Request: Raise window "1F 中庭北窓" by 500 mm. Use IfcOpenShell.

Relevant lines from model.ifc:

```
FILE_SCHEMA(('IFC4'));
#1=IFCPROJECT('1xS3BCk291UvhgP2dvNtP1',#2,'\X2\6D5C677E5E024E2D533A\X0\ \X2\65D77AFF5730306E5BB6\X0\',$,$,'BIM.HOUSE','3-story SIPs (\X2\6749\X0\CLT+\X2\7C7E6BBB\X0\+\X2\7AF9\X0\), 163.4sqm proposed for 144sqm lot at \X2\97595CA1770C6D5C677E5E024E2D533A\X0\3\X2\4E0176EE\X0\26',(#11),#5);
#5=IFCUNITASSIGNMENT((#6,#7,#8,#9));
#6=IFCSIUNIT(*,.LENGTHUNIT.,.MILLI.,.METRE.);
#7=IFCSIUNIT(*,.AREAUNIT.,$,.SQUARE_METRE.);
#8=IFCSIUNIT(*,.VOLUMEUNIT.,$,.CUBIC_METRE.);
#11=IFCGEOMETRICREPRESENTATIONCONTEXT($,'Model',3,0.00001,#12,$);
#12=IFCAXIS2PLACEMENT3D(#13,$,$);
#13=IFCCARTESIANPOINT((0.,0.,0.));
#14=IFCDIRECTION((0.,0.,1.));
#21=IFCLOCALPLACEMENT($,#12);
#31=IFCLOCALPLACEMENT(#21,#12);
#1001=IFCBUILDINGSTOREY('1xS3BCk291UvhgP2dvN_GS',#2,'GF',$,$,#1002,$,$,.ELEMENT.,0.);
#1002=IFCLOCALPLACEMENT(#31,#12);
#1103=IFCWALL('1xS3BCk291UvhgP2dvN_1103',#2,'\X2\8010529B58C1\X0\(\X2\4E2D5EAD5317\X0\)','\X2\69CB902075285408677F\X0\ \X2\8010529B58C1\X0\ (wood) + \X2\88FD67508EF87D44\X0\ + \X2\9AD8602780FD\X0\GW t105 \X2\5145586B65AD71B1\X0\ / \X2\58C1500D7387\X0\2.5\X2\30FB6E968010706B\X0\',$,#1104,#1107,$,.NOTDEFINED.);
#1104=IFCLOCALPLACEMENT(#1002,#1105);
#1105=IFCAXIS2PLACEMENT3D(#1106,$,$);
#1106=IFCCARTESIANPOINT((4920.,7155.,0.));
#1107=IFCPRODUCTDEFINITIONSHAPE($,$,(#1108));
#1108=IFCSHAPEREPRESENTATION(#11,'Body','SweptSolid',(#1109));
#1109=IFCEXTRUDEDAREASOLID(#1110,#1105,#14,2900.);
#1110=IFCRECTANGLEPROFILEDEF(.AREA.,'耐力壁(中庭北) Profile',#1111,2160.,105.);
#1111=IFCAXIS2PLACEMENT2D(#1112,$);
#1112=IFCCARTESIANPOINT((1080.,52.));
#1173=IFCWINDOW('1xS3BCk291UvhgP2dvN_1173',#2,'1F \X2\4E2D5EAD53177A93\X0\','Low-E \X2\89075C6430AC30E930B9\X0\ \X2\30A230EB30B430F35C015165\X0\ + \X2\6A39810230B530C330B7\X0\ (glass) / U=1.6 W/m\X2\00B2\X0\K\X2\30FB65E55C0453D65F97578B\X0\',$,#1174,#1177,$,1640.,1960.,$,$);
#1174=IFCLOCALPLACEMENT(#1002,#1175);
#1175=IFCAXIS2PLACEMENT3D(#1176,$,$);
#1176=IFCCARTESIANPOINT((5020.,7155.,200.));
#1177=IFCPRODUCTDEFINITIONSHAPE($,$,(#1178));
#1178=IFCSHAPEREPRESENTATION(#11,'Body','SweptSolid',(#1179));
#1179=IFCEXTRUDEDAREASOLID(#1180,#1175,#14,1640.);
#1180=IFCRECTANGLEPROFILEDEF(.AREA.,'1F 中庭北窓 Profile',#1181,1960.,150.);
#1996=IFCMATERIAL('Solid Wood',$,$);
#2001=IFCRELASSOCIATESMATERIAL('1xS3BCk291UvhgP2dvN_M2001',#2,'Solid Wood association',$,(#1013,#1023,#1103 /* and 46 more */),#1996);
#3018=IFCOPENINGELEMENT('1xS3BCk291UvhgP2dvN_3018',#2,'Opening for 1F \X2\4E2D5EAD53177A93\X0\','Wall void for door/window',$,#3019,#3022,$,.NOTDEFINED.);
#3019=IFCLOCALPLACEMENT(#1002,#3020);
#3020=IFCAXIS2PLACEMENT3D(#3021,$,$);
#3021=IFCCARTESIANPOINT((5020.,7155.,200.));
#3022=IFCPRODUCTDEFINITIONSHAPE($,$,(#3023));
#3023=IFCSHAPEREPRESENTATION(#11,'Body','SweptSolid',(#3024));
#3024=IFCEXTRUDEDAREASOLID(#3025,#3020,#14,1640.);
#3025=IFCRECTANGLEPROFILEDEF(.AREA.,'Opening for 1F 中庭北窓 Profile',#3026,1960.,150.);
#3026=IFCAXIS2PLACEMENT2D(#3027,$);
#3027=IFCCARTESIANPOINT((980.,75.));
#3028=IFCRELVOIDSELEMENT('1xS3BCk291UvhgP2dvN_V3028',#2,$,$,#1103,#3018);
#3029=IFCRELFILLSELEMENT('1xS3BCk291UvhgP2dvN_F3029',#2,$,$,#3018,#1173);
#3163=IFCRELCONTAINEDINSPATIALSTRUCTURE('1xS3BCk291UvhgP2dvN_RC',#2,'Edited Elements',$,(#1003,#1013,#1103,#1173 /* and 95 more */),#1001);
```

```python
import numpy as np
import ifcopenshell
import ifcopenshell.api.geometry
import ifcopenshell.util.placement
import ifcopenshell.util.unit

model = ifcopenshell.open("model.ifc")
unit_scale = ifcopenshell.util.unit.calculate_unit_scale(model)

window = model.by_guid("1xS3BCk291UvhgP2dvN_1173")
opening = window.FillsVoids[0].RelatingOpeningElement
dz = 0.5 / unit_scale

shift = np.array([0.0, 0.0, dz])
# The window is not placed relative to its opening, so move both.
for product in (opening, window):
    matrix = ifcopenshell.util.placement.get_local_placement(product.ObjectPlacement)
    matrix[:3, 3] += shift
    ifcopenshell.api.geometry.edit_object_placement(model, product=product, matrix=matrix, is_si=False)

print(f"moved by {dz * unit_scale:+.3f} m")

model.write("model_edited.ifc")
```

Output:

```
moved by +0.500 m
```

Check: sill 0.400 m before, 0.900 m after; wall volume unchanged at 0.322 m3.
